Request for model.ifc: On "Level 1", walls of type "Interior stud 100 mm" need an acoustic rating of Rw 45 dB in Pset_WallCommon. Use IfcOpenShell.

First a look at what the model holds.

```python
import ifcopenshell
import ifcopenshell.util.element

model = ifcopenshell.open("model.ifc")
print(model.schema)
storey = next(s for s in model.by_type("IfcBuildingStorey") if s.Name == "Level 1")
walls = [e for e in ifcopenshell.util.element.get_decomposition(storey) if e.is_a("IfcWall")]
seen = {}
for e in walls:
    element_type = ifcopenshell.util.element.get_type(e)
    key = (element_type.Name if element_type != e and element_type else None, ifcopenshell.util.element.get_pset(e, "Pset_WallCommon", "AcousticRating"))
    seen[key] = seen.get(key, 0) + 1
for (name, value), count in sorted(seen.items(), key=str):
    print(count, "x", name, "|", value)
```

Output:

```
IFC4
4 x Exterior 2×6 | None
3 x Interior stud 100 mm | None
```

```python
import ifcopenshell
import ifcopenshell.api.pset
import ifcopenshell.util.element

model = ifcopenshell.open("model.ifc")

storey = next(s for s in model.by_type("IfcBuildingStorey") if s.Name == "Level 1")
walls = [e for e in ifcopenshell.util.element.get_decomposition(storey) if e.is_a("IfcWall")]

count = 0
for e in walls:
    element_type = ifcopenshell.util.element.get_type(e)
    if element_type in (None, e) or element_type.Name != "Interior stud 100 mm":
        continue
    # add_pset returns the element's existing set when there is one.
    pset = ifcopenshell.api.pset.add_pset(model, product=e, name="Pset_WallCommon")
    ifcopenshell.api.pset.edit_pset(model, pset=pset, properties={"AcousticRating": "Rw 45 dB"})
    count += 1

print(count, "walls updated")

model.write("model_rev.ifc")
```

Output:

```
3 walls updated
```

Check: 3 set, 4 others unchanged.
